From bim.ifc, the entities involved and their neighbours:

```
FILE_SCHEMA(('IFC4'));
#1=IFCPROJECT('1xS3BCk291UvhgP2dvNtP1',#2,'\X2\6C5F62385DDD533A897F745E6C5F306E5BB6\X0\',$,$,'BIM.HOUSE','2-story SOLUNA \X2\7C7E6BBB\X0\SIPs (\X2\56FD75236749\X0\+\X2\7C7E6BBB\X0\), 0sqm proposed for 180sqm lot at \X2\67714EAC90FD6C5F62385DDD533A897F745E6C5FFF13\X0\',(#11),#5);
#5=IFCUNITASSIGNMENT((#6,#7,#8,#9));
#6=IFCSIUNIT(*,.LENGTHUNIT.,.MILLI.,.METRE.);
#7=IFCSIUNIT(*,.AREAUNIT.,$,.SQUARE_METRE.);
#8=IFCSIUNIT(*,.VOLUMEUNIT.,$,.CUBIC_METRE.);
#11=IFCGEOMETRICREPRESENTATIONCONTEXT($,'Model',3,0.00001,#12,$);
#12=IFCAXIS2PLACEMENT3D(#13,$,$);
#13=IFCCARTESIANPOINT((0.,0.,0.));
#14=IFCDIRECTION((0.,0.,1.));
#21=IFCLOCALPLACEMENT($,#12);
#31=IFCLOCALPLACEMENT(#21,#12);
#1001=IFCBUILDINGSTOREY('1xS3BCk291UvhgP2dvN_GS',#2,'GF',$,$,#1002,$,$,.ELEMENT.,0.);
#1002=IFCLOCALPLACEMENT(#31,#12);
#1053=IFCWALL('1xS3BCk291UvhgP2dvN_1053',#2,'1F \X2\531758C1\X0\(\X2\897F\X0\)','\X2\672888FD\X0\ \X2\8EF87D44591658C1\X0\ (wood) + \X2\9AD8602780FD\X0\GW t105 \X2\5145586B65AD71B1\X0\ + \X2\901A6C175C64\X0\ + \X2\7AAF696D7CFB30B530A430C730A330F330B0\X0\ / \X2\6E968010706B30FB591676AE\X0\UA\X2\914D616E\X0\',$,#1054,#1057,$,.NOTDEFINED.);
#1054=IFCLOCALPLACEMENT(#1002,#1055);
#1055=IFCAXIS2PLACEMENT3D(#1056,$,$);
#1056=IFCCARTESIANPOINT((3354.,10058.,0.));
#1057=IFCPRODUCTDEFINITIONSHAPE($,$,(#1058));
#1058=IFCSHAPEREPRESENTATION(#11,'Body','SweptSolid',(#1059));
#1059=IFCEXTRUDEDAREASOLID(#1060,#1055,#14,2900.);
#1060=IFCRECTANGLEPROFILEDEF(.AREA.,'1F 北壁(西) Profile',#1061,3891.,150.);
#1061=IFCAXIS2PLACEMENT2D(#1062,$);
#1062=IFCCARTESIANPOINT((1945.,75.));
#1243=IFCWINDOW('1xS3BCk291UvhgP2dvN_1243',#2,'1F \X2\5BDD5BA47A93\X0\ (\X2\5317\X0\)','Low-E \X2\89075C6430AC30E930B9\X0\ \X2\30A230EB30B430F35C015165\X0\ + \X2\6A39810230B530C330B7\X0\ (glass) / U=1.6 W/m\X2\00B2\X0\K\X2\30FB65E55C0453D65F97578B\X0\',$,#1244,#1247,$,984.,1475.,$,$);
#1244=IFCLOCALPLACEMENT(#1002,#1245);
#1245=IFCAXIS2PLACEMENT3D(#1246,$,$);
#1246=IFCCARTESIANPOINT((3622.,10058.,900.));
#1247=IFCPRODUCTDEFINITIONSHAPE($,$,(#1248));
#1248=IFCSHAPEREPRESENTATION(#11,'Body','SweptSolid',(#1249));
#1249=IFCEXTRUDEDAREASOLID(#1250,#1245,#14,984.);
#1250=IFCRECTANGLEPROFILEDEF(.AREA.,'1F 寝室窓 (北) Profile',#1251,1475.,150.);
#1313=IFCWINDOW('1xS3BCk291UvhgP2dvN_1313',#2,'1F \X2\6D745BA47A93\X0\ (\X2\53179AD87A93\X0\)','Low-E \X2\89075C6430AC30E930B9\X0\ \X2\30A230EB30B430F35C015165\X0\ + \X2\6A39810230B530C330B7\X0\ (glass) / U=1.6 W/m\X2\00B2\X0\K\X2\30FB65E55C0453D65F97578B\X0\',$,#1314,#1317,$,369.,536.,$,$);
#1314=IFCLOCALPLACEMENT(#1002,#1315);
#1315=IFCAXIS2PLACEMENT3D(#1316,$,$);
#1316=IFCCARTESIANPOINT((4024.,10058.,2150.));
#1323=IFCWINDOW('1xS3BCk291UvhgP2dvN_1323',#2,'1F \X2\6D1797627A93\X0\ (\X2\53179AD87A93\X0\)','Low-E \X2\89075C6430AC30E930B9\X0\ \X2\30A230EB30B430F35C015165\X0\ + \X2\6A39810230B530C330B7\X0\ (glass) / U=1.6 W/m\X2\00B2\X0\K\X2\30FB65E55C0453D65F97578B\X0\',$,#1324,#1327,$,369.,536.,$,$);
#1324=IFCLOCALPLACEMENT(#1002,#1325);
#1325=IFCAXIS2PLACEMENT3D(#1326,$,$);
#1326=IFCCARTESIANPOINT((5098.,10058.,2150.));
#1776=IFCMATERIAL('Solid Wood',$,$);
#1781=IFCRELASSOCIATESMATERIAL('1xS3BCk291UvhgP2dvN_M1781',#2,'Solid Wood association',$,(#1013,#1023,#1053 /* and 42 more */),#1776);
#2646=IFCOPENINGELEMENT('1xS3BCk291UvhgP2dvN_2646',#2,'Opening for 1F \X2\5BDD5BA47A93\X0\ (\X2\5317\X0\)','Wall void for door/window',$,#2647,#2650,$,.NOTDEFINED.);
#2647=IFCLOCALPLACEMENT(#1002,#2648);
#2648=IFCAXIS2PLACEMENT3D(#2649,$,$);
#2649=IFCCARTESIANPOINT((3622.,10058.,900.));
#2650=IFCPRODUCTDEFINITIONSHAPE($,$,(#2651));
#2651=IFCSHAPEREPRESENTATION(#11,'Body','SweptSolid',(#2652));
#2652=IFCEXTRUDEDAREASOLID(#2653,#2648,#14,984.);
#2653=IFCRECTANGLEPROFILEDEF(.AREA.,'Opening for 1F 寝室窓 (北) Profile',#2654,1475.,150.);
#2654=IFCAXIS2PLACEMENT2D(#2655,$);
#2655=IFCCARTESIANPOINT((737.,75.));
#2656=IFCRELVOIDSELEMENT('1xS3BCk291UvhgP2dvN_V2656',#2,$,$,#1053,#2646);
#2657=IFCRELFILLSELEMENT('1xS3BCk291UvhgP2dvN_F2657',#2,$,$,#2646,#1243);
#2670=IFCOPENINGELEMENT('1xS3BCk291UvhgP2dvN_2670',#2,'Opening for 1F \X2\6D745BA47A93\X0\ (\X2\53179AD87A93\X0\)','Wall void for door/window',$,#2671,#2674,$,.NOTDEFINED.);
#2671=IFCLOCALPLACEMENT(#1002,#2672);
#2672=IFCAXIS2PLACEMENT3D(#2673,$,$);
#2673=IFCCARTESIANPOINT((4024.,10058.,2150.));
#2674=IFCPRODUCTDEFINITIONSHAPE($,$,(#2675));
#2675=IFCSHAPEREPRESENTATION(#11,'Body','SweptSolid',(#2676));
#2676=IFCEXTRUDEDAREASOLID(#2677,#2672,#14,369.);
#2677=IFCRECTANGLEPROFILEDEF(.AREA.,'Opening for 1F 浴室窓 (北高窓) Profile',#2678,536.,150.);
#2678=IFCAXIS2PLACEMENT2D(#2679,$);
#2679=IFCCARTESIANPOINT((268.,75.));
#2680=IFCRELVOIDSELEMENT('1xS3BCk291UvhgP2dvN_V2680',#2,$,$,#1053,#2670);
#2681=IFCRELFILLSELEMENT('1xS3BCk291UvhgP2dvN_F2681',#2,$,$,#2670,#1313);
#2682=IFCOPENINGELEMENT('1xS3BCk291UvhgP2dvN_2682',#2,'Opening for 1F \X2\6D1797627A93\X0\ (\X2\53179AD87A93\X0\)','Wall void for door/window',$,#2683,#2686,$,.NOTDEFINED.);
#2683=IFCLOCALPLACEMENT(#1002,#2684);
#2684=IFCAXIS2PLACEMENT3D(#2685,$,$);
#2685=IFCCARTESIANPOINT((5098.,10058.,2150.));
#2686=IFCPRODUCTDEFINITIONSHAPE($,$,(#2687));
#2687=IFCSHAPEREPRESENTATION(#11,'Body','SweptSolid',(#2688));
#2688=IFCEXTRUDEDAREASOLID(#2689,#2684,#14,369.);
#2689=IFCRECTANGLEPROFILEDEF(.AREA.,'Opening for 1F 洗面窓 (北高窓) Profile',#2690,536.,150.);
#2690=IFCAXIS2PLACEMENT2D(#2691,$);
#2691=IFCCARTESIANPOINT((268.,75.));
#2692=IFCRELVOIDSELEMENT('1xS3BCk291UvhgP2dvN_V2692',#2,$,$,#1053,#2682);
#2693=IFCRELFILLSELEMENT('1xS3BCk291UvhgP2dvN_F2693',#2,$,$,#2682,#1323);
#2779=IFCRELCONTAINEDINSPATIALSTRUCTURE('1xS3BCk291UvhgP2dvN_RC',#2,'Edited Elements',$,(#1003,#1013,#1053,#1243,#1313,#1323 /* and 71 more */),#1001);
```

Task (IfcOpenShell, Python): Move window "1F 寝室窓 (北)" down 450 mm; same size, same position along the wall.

```python
import numpy as np
import ifcopenshell
import ifcopenshell.api.geometry
import ifcopenshell.util.placement
import ifcopenshell.util.unit

model = ifcopenshell.open("bim.ifc")
unit_scale = ifcopenshell.util.unit.calculate_unit_scale(model)

window = model.by_guid("1xS3BCk291UvhgP2dvN_1243")
opening = window.FillsVoids[0].RelatingOpeningElement
dz = -0.45 / unit_scale

shift = np.array([0.0, 0.0, dz])
# The window is not placed relative to its opening, so move both.
for product in (opening, window):
    matrix = ifcopenshell.util.placement.get_local_placement(product.ObjectPlacement)
    matrix[:3, 3] += shift
    ifcopenshell.api.geometry.edit_object_placement(model, product=product, matrix=matrix, is_si=False)

print(f"moved by {dz * unit_scale:+.3f} m")

model.write("bim_edited.ifc")
```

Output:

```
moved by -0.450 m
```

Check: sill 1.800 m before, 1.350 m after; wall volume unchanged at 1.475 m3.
